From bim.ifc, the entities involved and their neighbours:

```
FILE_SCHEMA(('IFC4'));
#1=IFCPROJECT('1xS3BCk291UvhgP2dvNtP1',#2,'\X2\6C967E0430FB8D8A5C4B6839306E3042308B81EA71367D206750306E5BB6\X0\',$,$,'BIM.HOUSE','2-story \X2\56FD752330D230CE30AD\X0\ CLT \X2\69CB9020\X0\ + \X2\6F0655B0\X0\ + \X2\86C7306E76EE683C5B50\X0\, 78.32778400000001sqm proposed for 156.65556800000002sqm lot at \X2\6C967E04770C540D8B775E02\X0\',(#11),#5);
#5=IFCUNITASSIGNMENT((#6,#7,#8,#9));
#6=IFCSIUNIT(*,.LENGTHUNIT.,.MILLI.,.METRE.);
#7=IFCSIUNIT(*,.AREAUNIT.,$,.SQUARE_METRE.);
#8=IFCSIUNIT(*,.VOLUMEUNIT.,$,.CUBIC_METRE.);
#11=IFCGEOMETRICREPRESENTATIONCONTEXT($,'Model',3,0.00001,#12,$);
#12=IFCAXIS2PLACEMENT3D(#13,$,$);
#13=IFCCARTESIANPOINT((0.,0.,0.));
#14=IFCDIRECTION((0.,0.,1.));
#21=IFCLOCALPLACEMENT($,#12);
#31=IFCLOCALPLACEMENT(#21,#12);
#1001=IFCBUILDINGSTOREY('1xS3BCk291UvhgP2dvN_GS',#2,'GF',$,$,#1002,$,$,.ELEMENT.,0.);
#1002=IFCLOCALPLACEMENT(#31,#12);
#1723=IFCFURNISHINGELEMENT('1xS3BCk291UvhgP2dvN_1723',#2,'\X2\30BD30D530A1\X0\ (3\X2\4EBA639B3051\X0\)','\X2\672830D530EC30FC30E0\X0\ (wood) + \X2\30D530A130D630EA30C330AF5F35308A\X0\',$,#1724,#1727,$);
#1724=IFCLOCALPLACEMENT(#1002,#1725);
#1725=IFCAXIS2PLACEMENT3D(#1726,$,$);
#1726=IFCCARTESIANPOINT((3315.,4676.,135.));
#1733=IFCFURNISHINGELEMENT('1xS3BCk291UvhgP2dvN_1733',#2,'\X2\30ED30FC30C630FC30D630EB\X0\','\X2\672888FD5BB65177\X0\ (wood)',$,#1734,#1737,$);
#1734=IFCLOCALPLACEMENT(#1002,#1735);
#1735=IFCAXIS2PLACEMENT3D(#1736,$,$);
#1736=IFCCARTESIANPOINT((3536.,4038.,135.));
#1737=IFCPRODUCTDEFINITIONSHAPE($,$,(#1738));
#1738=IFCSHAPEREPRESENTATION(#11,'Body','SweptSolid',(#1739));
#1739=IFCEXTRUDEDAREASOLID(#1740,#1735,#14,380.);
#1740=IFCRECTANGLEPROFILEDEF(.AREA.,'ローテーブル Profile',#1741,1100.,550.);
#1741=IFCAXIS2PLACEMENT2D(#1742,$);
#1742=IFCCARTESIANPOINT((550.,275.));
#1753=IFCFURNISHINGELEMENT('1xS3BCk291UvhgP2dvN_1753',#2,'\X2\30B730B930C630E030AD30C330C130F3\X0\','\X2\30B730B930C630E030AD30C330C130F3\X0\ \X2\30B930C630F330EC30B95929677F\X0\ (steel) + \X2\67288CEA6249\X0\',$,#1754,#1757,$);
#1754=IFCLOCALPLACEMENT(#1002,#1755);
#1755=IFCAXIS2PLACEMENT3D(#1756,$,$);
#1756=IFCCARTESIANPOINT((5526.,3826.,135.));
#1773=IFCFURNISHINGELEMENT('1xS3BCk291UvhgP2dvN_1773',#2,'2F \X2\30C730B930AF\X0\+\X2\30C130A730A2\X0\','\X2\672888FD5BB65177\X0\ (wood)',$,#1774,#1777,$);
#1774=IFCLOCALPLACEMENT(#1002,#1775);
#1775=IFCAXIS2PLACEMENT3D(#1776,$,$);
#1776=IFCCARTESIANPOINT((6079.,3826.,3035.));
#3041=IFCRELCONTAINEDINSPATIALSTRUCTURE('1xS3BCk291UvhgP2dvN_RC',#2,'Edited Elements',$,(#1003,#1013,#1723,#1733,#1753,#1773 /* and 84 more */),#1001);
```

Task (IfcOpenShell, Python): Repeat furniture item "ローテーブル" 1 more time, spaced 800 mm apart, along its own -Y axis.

```python
import ifcopenshell
import ifcopenshell.api.geometry
import ifcopenshell.api.root
import ifcopenshell.util.element
import ifcopenshell.util.placement

model = ifcopenshell.open("bim.ifc")


def reuse_history(source, copy):
    """copy_class also copies each property set's owner history, people and application; keep the originals."""
    for rel in copy.IsDefinedBy:
        if rel.is_a("IfcRelDefinesByProperties") and (history := rel.RelatingPropertyDefinition.OwnerHistory):
            rel.RelatingPropertyDefinition.OwnerHistory = source.OwnerHistory
            ifcopenshell.util.element.remove_deep2(model, history)


source = model.by_guid("1xS3BCk291UvhgP2dvN_1733")
base = ifcopenshell.util.placement.get_local_placement(source.ObjectPlacement)
step = -base[:3, 1] * 800.0

for i in range(1, 2):
    copy = ifcopenshell.api.root.copy_class(model, product=source)
    copy.Representation = ifcopenshell.util.element.copy_deep(
        model, source.Representation, exclude=["IfcGeometricRepresentationContext", "IfcRepresentationMap"]
    )
    reuse_history(source, copy)
    matrix = base.copy()
    matrix[:3, 3] += i * step
    print("added at", matrix[:3, 3].round(3) + 0.0)
    ifcopenshell.api.geometry.edit_object_placement(model, product=copy, matrix=matrix, is_si=False)

model.write("bim_v2.ifc")
```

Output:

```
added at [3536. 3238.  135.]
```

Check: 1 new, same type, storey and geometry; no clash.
